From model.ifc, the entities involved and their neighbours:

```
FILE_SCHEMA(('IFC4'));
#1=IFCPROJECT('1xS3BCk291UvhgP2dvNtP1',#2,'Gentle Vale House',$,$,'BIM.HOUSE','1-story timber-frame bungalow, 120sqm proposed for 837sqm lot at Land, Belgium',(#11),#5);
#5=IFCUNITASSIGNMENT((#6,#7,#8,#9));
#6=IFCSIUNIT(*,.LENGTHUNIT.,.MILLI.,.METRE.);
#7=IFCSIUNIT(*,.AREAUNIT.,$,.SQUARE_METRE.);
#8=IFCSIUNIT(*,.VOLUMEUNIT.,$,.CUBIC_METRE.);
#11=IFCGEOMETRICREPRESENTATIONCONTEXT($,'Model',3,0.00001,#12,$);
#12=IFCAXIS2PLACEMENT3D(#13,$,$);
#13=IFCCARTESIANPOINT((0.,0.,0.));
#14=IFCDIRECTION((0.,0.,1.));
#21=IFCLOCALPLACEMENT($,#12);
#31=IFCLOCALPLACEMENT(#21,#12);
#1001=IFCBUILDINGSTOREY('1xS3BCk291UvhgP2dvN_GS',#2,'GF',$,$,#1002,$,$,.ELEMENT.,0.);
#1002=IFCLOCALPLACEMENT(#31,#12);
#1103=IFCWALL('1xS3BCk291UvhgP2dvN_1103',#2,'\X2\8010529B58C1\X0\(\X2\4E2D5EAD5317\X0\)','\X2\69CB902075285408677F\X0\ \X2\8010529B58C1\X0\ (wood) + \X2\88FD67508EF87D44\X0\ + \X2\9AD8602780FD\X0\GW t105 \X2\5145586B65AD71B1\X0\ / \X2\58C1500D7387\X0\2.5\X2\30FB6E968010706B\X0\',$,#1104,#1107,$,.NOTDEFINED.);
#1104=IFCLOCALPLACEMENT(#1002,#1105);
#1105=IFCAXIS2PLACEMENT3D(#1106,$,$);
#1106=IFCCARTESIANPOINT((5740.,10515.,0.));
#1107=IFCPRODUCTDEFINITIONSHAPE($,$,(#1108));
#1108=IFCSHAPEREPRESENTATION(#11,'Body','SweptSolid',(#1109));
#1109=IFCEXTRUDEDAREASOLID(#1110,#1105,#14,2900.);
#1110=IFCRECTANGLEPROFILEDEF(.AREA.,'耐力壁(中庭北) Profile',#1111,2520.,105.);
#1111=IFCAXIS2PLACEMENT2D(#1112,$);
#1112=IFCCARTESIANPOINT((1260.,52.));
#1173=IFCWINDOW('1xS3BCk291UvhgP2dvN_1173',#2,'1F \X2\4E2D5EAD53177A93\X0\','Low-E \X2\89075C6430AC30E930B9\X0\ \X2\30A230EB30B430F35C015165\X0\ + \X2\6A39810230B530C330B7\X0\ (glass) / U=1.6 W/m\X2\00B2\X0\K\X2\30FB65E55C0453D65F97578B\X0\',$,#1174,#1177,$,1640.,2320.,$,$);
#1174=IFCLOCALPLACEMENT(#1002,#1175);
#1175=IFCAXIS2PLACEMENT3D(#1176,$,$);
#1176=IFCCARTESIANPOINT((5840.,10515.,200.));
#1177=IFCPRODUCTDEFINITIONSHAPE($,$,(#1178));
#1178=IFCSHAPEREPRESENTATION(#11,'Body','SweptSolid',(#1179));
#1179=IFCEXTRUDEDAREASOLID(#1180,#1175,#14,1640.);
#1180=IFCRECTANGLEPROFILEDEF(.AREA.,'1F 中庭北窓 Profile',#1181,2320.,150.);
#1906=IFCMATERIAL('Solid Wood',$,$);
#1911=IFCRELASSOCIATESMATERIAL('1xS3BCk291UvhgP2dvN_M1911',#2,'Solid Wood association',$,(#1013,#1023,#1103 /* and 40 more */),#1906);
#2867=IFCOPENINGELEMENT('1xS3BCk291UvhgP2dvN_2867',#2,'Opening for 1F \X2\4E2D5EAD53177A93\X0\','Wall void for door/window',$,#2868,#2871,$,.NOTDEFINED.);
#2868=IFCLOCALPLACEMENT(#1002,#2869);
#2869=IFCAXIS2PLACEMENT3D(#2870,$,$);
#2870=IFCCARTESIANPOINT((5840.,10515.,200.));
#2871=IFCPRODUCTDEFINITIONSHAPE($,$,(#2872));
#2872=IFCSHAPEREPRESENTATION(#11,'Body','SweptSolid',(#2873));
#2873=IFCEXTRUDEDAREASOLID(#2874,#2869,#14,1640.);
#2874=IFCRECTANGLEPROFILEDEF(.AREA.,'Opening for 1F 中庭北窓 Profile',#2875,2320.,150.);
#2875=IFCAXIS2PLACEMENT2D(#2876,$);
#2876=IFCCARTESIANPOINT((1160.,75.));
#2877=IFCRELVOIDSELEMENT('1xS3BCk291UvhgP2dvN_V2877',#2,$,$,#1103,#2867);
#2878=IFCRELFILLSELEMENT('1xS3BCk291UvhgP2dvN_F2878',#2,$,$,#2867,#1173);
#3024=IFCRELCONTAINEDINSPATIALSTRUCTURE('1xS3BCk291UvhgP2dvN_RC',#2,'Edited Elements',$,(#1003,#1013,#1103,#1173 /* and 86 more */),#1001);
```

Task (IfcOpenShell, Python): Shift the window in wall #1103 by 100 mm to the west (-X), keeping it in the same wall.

```python
import ifcopenshell
import ifcopenshell.api.geometry
import ifcopenshell.util.placement
import ifcopenshell.util.unit

model = ifcopenshell.open("model.ifc")
unit_scale = ifcopenshell.util.unit.calculate_unit_scale(model)

window = model.by_guid("1xS3BCk291UvhgP2dvN_1173")
opening = window.FillsVoids[0].RelatingOpeningElement
wall = opening.VoidsElements[0].RelatingBuildingElement

wall_matrix = ifcopenshell.util.placement.get_local_placement(wall.ObjectPlacement)
shift = wall_matrix[:3, 0] * -0.1 / unit_scale
before = ifcopenshell.util.placement.get_local_placement(window.ObjectPlacement)[:3, 3].copy()

# The window is not placed relative to its opening, so move both.
for product in (opening, window):
    matrix = ifcopenshell.util.placement.get_local_placement(product.ObjectPlacement)
    matrix[:3, 3] += shift
    ifcopenshell.api.geometry.edit_object_placement(model, product=product, matrix=matrix, is_si=False)

after = ifcopenshell.util.placement.get_local_placement(window.ObjectPlacement)[:3, 3]
print("window moved by", (after - before).round(3) + 0.0)

model.write("model-out.ifc")
```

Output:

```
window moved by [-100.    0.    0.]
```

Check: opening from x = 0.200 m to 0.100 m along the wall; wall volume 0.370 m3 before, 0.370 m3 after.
